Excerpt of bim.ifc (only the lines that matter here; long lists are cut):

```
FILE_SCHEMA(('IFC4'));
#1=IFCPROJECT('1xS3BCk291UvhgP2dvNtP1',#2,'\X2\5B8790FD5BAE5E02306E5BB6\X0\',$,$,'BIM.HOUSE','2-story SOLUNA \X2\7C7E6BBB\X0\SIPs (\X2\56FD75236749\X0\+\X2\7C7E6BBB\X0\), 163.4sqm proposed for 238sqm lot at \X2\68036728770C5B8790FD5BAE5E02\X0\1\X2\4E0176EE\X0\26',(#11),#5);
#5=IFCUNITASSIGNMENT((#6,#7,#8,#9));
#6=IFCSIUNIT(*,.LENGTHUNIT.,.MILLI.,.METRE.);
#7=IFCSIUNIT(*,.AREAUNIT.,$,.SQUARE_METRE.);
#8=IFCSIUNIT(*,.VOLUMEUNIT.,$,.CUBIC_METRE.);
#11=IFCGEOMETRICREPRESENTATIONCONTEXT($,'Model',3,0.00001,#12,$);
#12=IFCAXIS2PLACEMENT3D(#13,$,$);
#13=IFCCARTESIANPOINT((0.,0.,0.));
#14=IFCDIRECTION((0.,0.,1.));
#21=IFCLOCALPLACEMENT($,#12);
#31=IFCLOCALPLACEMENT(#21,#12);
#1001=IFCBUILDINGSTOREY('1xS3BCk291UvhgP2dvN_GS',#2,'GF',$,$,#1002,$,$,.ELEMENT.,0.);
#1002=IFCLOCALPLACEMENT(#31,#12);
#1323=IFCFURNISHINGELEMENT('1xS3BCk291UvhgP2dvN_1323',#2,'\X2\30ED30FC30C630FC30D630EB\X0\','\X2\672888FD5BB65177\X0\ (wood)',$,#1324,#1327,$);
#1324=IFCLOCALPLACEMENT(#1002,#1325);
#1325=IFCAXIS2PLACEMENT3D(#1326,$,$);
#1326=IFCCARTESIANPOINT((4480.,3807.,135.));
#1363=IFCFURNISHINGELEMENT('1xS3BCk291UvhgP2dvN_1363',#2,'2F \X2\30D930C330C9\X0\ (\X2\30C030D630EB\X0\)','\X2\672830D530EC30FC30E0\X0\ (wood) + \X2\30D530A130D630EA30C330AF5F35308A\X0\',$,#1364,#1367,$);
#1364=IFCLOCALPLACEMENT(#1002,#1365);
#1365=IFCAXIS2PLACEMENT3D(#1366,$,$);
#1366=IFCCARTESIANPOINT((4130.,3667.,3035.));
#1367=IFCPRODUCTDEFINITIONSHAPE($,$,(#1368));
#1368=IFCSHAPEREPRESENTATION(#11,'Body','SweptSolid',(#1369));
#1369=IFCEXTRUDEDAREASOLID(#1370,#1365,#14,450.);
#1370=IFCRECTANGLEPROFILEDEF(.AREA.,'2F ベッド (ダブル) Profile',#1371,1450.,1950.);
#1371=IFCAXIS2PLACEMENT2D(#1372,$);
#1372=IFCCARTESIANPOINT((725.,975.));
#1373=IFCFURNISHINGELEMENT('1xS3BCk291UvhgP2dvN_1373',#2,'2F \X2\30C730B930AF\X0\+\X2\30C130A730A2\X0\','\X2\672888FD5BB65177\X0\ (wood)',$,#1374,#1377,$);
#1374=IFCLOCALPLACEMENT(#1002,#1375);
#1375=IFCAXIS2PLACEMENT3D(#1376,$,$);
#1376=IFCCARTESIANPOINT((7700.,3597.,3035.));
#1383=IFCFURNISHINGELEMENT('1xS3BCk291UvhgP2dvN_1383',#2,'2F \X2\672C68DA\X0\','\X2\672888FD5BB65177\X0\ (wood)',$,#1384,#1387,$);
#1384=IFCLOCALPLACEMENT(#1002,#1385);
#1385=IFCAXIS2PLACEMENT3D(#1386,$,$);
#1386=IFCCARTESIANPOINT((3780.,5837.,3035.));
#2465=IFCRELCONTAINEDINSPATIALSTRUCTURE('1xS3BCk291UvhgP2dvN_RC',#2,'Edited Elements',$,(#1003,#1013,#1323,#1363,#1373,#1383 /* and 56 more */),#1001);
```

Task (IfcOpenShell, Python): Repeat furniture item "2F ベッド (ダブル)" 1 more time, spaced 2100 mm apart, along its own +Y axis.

```python
import ifcopenshell
import ifcopenshell.api.geometry
import ifcopenshell.api.root
import ifcopenshell.util.element
import ifcopenshell.util.placement
import ifcopenshell.util.unit

model = ifcopenshell.open("bim.ifc")
unit_scale = ifcopenshell.util.unit.calculate_unit_scale(model)


def reuse_history(source, copy):
    """copy_class also copies each property set's owner history, people and application; keep the originals."""
    for rel in copy.IsDefinedBy:
        if rel.is_a("IfcRelDefinesByProperties") and (history := rel.RelatingPropertyDefinition.OwnerHistory):
            rel.RelatingPropertyDefinition.OwnerHistory = source.OwnerHistory
            ifcopenshell.util.element.remove_deep2(model, history)


source = model.by_guid("1xS3BCk291UvhgP2dvN_1363")
base = ifcopenshell.util.placement.get_local_placement(source.ObjectPlacement)
step = base[:3, 1] * 2.1 / unit_scale

for i in range(1, 2):
    copy = ifcopenshell.api.root.copy_class(model, product=source)
    copy.Representation = ifcopenshell.util.element.copy_deep(
        model, source.Representation, exclude=["IfcGeometricRepresentationContext", "IfcRepresentationMap"]
    )
    reuse_history(source, copy)
    matrix = base.copy()
    matrix[:3, 3] += i * step
    print("added at", matrix[:3, 3].round(3) + 0.0)
    ifcopenshell.api.geometry.edit_object_placement(model, product=copy, matrix=matrix, is_si=False)

model.write("bim_rev.ifc")
```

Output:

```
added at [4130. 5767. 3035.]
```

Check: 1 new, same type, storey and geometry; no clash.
